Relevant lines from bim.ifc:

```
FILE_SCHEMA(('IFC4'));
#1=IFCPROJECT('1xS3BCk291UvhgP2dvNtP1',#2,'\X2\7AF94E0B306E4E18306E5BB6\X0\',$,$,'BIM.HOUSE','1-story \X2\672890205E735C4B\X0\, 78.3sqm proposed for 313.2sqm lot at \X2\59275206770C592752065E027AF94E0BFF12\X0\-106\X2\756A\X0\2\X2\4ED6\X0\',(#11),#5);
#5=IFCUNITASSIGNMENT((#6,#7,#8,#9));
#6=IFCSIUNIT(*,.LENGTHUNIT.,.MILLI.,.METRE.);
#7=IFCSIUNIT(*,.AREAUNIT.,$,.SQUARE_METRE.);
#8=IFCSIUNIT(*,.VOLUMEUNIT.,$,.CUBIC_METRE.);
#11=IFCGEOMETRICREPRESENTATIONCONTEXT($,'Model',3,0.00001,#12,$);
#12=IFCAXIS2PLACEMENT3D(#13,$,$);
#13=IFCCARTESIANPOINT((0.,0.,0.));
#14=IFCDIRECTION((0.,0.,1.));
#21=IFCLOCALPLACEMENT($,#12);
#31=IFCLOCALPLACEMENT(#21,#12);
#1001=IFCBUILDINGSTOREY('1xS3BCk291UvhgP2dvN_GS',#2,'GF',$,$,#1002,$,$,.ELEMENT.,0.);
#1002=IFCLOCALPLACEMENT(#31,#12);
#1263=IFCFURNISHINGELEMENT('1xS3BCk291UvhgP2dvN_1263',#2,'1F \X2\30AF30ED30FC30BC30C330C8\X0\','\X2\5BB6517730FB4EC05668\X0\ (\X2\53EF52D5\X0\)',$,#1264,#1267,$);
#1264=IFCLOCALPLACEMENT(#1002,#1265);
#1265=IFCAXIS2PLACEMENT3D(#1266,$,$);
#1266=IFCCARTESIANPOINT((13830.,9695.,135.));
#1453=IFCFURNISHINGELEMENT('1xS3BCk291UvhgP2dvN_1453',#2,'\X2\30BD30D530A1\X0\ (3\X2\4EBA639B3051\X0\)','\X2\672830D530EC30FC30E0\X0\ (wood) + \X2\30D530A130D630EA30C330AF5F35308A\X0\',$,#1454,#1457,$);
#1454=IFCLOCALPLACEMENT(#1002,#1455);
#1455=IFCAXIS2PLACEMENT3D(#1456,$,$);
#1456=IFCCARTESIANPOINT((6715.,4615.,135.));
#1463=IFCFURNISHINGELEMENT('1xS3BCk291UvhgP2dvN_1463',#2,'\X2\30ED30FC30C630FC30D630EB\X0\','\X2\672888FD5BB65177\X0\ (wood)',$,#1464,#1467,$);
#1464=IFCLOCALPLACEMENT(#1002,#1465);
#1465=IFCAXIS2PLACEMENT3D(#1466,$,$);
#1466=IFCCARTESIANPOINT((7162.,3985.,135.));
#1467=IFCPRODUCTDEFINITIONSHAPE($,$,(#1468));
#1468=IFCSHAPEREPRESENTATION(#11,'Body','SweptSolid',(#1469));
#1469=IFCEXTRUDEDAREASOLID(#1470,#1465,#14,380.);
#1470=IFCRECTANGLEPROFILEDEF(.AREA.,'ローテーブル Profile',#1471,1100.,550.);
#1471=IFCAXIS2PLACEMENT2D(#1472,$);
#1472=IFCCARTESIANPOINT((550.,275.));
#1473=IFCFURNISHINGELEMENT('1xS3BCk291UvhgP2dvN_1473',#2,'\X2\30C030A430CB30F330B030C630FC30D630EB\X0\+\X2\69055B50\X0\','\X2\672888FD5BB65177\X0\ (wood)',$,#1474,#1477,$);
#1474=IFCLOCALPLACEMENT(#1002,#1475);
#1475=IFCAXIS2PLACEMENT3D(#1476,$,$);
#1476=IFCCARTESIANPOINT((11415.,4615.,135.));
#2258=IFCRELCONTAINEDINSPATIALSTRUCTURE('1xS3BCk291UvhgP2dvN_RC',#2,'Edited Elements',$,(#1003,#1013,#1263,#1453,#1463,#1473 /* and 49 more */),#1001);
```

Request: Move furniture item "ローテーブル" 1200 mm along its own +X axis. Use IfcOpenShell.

```python
import ifcopenshell
import ifcopenshell.api.geometry
import ifcopenshell.util.placement

model = ifcopenshell.open("bim.ifc")

item = model.by_guid("1xS3BCk291UvhgP2dvN_1463")
matrix = ifcopenshell.util.placement.get_local_placement(item.ObjectPlacement)
matrix[:3, 3] += matrix[:3, 0] * 1200.0
ifcopenshell.api.geometry.edit_object_placement(model, product=item, matrix=matrix, is_si=False)

print(ifcopenshell.util.placement.get_local_placement(item.ObjectPlacement).round(3) + 0.0)

model.write("bim_updated.ifc")
```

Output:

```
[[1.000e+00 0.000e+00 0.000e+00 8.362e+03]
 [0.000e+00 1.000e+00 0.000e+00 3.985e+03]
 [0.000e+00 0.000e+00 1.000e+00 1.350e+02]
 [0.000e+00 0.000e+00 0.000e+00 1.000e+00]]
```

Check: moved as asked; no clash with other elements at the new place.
